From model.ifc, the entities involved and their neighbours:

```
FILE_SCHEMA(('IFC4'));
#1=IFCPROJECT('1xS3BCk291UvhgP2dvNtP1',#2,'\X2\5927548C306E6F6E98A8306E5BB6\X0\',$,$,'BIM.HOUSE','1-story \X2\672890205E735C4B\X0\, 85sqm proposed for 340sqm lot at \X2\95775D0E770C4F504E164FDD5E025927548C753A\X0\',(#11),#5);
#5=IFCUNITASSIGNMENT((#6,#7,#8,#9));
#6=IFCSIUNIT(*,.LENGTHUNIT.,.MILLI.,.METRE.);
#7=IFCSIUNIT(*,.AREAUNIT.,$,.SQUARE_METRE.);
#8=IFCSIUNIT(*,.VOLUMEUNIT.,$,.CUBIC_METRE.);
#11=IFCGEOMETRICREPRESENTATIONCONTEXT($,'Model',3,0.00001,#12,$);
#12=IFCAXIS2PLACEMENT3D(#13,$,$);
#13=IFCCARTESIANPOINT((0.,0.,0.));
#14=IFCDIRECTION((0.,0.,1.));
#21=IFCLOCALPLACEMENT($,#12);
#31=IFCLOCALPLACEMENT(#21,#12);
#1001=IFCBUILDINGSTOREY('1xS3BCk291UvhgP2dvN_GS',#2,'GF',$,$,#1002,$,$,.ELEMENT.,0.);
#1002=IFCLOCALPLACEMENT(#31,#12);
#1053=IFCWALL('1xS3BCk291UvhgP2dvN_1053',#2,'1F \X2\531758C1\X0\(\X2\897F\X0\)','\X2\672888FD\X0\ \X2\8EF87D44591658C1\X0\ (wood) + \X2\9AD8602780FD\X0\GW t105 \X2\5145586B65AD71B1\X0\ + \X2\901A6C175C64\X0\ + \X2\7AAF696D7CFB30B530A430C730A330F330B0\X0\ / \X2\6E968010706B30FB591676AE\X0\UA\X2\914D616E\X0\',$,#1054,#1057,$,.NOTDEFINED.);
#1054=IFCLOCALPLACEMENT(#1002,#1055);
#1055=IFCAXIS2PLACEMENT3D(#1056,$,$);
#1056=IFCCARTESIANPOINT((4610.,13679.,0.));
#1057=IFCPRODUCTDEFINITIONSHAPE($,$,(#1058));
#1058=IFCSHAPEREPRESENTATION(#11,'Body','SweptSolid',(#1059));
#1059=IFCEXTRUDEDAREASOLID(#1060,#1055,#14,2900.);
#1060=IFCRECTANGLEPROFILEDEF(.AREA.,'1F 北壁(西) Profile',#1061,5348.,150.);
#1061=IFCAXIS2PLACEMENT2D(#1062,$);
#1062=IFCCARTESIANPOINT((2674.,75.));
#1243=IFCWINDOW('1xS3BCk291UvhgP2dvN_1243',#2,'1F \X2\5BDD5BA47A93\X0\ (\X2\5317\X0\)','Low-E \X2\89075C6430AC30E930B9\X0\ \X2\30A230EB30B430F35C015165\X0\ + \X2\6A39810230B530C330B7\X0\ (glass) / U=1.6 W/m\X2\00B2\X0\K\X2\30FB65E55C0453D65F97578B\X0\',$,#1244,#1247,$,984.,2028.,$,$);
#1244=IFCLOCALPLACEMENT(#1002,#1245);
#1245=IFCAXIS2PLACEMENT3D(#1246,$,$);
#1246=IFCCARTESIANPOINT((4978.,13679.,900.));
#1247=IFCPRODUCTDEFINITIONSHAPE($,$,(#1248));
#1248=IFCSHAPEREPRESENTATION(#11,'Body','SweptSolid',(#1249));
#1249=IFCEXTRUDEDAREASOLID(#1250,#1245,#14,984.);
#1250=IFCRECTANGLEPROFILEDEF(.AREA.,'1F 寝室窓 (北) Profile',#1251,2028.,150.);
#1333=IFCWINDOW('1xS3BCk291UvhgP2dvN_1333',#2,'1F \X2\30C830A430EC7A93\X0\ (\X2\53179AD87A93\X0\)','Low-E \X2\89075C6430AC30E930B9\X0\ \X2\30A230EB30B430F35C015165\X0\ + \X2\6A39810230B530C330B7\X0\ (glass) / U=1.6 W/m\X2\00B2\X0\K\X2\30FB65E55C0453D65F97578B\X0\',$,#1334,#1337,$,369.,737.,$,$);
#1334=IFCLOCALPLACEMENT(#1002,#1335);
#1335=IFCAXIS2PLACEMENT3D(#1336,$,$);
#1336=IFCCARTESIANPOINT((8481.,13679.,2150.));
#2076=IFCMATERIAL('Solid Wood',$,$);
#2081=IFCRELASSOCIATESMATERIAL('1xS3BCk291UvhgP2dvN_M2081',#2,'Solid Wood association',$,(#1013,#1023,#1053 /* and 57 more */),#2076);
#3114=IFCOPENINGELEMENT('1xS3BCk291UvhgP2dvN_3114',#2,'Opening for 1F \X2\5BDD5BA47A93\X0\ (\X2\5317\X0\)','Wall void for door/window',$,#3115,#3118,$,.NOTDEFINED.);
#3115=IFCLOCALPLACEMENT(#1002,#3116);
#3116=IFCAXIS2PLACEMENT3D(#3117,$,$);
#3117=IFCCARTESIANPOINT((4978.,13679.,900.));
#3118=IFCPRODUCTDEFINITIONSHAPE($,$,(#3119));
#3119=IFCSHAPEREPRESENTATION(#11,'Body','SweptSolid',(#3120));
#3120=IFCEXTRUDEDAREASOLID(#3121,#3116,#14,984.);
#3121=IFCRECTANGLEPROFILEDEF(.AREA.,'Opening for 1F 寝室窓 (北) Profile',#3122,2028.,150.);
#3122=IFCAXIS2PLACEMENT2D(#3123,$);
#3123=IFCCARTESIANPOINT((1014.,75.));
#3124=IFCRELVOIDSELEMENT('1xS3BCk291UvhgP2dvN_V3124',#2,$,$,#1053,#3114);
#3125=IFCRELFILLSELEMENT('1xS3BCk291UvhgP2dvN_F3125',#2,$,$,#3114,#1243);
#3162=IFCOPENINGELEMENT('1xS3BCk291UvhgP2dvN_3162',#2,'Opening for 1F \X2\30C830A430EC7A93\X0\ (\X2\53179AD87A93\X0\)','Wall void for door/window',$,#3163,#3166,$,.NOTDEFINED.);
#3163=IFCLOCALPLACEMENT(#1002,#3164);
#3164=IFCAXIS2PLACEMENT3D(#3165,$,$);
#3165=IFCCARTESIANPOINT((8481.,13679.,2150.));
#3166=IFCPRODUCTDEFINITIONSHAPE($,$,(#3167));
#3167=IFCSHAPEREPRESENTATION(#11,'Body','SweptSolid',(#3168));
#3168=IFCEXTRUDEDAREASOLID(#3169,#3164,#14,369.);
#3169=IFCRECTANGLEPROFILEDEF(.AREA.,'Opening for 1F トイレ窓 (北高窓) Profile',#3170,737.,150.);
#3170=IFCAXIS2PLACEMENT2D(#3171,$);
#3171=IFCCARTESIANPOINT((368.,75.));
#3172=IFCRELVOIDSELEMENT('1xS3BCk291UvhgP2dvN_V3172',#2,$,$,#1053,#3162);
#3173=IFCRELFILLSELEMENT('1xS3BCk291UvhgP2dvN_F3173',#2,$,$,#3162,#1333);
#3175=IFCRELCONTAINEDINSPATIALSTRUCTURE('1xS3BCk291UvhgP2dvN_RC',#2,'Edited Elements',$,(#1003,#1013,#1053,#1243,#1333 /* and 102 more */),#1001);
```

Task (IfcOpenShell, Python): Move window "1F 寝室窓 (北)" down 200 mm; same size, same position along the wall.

```python
import numpy as np
import ifcopenshell
import ifcopenshell.api.geometry
import ifcopenshell.util.placement
import ifcopenshell.util.unit

model = ifcopenshell.open("model.ifc")
unit_scale = ifcopenshell.util.unit.calculate_unit_scale(model)

window = model.by_guid("1xS3BCk291UvhgP2dvN_1243")
opening = window.FillsVoids[0].RelatingOpeningElement
dz = -0.2 / unit_scale

shift = np.array([0.0, 0.0, dz])
# The window is not placed relative to its opening, so move both.
for product in (opening, window):
    matrix = ifcopenshell.util.placement.get_local_placement(product.ObjectPlacement)
    matrix[:3, 3] += shift
    ifcopenshell.api.geometry.edit_object_placement(model, product=product, matrix=matrix, is_si=False)

print(f"moved by {dz * unit_scale:+.3f} m")

model.write("model-out.ifc")
```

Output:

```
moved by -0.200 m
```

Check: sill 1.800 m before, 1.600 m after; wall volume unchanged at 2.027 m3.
